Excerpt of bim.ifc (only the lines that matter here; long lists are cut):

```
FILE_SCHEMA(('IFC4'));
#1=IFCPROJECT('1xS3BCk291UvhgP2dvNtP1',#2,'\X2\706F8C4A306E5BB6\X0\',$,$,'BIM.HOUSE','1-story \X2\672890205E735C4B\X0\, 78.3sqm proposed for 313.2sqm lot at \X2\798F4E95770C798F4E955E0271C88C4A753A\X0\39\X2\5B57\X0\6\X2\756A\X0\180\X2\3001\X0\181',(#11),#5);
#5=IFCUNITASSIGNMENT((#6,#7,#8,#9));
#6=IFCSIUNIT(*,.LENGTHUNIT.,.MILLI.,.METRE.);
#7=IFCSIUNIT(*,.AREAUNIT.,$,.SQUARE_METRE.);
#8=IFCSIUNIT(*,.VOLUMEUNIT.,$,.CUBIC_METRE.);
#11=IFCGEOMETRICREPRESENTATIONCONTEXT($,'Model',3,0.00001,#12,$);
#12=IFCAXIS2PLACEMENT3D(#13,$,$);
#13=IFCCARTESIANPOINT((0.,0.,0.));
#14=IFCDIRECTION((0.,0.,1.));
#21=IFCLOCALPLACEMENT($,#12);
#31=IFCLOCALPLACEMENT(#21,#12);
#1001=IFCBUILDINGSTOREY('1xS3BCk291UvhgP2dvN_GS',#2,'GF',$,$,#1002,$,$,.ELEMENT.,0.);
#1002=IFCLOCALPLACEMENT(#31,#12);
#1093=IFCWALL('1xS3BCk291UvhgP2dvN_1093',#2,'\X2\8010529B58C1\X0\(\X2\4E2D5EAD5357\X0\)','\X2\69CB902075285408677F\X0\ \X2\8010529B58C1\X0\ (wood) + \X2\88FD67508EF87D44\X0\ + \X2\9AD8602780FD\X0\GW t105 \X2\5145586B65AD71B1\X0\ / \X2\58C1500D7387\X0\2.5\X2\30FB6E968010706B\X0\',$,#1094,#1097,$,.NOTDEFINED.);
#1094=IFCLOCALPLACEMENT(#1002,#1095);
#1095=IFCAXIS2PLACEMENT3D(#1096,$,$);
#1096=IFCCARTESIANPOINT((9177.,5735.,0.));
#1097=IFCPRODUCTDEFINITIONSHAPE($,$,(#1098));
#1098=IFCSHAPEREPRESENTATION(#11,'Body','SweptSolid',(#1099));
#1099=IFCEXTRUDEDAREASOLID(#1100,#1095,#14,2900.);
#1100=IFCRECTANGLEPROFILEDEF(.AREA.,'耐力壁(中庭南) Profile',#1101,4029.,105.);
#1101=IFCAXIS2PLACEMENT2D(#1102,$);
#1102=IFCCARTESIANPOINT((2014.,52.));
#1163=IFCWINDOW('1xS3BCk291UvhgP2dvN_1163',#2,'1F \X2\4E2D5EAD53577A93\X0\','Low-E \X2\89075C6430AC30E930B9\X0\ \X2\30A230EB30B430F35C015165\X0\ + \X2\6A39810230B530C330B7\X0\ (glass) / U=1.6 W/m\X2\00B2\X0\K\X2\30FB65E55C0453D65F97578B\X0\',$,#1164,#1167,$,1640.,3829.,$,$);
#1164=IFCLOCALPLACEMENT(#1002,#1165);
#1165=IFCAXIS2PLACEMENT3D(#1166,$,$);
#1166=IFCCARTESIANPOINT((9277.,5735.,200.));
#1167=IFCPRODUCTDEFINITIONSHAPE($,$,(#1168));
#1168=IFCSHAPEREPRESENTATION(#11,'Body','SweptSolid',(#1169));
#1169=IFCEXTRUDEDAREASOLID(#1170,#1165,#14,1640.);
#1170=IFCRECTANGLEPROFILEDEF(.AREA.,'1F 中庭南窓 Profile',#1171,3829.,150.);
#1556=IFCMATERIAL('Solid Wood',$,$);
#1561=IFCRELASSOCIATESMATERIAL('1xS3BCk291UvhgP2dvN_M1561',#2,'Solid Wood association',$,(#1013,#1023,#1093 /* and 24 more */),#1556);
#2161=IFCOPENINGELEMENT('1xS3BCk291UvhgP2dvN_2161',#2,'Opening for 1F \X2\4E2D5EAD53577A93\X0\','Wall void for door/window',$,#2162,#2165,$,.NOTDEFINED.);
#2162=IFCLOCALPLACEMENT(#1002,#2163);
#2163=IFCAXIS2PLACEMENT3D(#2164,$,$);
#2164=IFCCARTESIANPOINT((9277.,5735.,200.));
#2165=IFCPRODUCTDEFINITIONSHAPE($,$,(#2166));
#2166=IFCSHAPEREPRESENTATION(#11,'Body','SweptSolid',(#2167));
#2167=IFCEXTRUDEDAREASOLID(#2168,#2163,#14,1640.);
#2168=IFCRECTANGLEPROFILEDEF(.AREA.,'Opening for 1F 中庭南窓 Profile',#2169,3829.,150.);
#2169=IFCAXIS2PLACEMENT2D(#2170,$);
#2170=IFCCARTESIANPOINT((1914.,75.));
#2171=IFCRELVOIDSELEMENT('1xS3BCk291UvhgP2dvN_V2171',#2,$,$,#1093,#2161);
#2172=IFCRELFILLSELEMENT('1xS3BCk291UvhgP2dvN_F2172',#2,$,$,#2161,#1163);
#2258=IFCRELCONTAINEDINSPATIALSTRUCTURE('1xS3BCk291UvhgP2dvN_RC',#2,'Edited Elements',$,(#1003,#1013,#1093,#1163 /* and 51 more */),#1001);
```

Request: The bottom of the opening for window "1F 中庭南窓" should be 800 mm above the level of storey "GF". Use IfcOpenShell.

```python
import numpy as np
import ifcopenshell
import ifcopenshell.api.geometry
import ifcopenshell.geom
import ifcopenshell.util.element
import ifcopenshell.util.placement
import ifcopenshell.util.shape
import ifcopenshell.util.unit

model = ifcopenshell.open("bim.ifc")
unit_scale = ifcopenshell.util.unit.calculate_unit_scale(model)

window = model.by_guid("1xS3BCk291UvhgP2dvN_1163")
opening = window.FillsVoids[0].RelatingOpeningElement
storey = ifcopenshell.util.element.get_container(window, ifc_class="IfcBuildingStorey")
level = ifcopenshell.util.placement.get_local_placement(storey.ObjectPlacement)[2, 3]

# The opening's origin need not be at the sill, so measure its lowest point.
shape = ifcopenshell.geom.create_shape(ifcopenshell.geom.settings(), opening)
bottom = ifcopenshell.util.shape.get_shape_bottom_elevation(shape, shape.geometry) / unit_scale
dz = level + 0.8 / unit_scale - bottom

shift = np.array([0.0, 0.0, dz])
# The window is not placed relative to its opening, so move both.
for product in (opening, window):
    matrix = ifcopenshell.util.placement.get_local_placement(product.ObjectPlacement)
    matrix[:3, 3] += shift
    ifcopenshell.api.geometry.edit_object_placement(model, product=product, matrix=matrix, is_si=False)

print(f"moved by {dz * unit_scale:+.3f} m")

model.write("bim_v2.ifc")
```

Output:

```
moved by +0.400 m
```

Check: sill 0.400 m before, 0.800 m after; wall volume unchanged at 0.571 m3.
